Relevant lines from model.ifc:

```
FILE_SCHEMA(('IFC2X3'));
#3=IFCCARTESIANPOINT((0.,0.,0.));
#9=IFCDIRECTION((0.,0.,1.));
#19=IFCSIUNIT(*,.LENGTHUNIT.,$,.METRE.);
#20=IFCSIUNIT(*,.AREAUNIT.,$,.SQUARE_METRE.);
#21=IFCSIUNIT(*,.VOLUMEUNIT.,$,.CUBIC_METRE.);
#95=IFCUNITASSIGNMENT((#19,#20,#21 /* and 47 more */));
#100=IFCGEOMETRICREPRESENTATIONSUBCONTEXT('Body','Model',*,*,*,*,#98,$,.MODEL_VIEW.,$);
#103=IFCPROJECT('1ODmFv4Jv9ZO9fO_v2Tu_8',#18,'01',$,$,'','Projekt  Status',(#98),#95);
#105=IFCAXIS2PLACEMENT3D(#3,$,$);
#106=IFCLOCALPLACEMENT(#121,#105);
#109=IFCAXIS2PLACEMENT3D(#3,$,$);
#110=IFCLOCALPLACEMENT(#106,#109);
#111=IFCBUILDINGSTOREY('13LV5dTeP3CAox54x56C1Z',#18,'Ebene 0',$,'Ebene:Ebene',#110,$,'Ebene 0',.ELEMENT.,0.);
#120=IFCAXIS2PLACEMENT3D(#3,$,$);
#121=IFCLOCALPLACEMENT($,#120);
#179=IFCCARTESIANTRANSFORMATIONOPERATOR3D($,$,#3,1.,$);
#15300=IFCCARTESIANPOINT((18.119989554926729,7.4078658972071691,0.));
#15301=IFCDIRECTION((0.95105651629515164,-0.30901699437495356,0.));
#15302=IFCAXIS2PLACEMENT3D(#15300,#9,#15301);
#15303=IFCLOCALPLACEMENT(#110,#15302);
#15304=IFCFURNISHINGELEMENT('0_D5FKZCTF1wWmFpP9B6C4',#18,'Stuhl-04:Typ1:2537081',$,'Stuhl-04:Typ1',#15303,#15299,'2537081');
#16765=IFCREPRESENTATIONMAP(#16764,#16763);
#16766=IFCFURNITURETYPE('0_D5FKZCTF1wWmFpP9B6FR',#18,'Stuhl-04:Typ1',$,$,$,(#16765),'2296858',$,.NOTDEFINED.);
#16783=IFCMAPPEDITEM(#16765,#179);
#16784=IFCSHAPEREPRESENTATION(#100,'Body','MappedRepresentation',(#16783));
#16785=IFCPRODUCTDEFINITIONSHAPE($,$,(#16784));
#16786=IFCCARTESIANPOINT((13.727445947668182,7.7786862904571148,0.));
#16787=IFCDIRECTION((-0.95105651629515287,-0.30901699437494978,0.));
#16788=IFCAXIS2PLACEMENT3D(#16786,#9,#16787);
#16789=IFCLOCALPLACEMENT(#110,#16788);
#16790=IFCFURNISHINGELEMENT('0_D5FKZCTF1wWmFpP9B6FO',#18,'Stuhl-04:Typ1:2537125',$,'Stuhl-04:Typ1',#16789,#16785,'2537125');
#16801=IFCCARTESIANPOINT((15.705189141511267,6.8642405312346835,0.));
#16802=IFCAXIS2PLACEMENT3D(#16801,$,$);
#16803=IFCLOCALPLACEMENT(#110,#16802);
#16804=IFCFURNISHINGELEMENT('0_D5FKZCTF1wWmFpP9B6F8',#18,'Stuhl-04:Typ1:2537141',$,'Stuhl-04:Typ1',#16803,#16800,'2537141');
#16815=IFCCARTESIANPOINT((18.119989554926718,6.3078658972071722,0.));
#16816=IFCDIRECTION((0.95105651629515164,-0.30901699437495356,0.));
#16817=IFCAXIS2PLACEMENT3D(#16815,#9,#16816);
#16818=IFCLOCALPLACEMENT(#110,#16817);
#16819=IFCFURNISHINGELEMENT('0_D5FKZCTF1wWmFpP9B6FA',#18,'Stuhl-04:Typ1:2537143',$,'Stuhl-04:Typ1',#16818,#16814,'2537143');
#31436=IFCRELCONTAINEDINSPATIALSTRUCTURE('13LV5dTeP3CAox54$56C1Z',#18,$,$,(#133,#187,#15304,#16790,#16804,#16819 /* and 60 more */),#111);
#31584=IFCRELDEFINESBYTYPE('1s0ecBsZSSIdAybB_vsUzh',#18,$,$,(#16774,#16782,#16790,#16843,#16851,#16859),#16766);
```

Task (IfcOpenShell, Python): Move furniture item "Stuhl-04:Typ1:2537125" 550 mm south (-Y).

```python
import ifcopenshell
import ifcopenshell.api.geometry
import ifcopenshell.util.placement
import ifcopenshell.util.unit

model = ifcopenshell.open("model.ifc")
unit_scale = ifcopenshell.util.unit.calculate_unit_scale(model)

item = model.by_guid("0_D5FKZCTF1wWmFpP9B6FO")
matrix = ifcopenshell.util.placement.get_local_placement(item.ObjectPlacement)
matrix[1, 3] -= 0.55 / unit_scale
ifcopenshell.api.geometry.edit_object_placement(model, product=item, matrix=matrix, is_si=False)

print(ifcopenshell.util.placement.get_local_placement(item.ObjectPlacement).round(3) + 0.0)

model.write("model-out.ifc")
```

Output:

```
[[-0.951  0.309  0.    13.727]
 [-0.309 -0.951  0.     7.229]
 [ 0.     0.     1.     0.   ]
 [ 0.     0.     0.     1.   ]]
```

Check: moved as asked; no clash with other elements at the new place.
